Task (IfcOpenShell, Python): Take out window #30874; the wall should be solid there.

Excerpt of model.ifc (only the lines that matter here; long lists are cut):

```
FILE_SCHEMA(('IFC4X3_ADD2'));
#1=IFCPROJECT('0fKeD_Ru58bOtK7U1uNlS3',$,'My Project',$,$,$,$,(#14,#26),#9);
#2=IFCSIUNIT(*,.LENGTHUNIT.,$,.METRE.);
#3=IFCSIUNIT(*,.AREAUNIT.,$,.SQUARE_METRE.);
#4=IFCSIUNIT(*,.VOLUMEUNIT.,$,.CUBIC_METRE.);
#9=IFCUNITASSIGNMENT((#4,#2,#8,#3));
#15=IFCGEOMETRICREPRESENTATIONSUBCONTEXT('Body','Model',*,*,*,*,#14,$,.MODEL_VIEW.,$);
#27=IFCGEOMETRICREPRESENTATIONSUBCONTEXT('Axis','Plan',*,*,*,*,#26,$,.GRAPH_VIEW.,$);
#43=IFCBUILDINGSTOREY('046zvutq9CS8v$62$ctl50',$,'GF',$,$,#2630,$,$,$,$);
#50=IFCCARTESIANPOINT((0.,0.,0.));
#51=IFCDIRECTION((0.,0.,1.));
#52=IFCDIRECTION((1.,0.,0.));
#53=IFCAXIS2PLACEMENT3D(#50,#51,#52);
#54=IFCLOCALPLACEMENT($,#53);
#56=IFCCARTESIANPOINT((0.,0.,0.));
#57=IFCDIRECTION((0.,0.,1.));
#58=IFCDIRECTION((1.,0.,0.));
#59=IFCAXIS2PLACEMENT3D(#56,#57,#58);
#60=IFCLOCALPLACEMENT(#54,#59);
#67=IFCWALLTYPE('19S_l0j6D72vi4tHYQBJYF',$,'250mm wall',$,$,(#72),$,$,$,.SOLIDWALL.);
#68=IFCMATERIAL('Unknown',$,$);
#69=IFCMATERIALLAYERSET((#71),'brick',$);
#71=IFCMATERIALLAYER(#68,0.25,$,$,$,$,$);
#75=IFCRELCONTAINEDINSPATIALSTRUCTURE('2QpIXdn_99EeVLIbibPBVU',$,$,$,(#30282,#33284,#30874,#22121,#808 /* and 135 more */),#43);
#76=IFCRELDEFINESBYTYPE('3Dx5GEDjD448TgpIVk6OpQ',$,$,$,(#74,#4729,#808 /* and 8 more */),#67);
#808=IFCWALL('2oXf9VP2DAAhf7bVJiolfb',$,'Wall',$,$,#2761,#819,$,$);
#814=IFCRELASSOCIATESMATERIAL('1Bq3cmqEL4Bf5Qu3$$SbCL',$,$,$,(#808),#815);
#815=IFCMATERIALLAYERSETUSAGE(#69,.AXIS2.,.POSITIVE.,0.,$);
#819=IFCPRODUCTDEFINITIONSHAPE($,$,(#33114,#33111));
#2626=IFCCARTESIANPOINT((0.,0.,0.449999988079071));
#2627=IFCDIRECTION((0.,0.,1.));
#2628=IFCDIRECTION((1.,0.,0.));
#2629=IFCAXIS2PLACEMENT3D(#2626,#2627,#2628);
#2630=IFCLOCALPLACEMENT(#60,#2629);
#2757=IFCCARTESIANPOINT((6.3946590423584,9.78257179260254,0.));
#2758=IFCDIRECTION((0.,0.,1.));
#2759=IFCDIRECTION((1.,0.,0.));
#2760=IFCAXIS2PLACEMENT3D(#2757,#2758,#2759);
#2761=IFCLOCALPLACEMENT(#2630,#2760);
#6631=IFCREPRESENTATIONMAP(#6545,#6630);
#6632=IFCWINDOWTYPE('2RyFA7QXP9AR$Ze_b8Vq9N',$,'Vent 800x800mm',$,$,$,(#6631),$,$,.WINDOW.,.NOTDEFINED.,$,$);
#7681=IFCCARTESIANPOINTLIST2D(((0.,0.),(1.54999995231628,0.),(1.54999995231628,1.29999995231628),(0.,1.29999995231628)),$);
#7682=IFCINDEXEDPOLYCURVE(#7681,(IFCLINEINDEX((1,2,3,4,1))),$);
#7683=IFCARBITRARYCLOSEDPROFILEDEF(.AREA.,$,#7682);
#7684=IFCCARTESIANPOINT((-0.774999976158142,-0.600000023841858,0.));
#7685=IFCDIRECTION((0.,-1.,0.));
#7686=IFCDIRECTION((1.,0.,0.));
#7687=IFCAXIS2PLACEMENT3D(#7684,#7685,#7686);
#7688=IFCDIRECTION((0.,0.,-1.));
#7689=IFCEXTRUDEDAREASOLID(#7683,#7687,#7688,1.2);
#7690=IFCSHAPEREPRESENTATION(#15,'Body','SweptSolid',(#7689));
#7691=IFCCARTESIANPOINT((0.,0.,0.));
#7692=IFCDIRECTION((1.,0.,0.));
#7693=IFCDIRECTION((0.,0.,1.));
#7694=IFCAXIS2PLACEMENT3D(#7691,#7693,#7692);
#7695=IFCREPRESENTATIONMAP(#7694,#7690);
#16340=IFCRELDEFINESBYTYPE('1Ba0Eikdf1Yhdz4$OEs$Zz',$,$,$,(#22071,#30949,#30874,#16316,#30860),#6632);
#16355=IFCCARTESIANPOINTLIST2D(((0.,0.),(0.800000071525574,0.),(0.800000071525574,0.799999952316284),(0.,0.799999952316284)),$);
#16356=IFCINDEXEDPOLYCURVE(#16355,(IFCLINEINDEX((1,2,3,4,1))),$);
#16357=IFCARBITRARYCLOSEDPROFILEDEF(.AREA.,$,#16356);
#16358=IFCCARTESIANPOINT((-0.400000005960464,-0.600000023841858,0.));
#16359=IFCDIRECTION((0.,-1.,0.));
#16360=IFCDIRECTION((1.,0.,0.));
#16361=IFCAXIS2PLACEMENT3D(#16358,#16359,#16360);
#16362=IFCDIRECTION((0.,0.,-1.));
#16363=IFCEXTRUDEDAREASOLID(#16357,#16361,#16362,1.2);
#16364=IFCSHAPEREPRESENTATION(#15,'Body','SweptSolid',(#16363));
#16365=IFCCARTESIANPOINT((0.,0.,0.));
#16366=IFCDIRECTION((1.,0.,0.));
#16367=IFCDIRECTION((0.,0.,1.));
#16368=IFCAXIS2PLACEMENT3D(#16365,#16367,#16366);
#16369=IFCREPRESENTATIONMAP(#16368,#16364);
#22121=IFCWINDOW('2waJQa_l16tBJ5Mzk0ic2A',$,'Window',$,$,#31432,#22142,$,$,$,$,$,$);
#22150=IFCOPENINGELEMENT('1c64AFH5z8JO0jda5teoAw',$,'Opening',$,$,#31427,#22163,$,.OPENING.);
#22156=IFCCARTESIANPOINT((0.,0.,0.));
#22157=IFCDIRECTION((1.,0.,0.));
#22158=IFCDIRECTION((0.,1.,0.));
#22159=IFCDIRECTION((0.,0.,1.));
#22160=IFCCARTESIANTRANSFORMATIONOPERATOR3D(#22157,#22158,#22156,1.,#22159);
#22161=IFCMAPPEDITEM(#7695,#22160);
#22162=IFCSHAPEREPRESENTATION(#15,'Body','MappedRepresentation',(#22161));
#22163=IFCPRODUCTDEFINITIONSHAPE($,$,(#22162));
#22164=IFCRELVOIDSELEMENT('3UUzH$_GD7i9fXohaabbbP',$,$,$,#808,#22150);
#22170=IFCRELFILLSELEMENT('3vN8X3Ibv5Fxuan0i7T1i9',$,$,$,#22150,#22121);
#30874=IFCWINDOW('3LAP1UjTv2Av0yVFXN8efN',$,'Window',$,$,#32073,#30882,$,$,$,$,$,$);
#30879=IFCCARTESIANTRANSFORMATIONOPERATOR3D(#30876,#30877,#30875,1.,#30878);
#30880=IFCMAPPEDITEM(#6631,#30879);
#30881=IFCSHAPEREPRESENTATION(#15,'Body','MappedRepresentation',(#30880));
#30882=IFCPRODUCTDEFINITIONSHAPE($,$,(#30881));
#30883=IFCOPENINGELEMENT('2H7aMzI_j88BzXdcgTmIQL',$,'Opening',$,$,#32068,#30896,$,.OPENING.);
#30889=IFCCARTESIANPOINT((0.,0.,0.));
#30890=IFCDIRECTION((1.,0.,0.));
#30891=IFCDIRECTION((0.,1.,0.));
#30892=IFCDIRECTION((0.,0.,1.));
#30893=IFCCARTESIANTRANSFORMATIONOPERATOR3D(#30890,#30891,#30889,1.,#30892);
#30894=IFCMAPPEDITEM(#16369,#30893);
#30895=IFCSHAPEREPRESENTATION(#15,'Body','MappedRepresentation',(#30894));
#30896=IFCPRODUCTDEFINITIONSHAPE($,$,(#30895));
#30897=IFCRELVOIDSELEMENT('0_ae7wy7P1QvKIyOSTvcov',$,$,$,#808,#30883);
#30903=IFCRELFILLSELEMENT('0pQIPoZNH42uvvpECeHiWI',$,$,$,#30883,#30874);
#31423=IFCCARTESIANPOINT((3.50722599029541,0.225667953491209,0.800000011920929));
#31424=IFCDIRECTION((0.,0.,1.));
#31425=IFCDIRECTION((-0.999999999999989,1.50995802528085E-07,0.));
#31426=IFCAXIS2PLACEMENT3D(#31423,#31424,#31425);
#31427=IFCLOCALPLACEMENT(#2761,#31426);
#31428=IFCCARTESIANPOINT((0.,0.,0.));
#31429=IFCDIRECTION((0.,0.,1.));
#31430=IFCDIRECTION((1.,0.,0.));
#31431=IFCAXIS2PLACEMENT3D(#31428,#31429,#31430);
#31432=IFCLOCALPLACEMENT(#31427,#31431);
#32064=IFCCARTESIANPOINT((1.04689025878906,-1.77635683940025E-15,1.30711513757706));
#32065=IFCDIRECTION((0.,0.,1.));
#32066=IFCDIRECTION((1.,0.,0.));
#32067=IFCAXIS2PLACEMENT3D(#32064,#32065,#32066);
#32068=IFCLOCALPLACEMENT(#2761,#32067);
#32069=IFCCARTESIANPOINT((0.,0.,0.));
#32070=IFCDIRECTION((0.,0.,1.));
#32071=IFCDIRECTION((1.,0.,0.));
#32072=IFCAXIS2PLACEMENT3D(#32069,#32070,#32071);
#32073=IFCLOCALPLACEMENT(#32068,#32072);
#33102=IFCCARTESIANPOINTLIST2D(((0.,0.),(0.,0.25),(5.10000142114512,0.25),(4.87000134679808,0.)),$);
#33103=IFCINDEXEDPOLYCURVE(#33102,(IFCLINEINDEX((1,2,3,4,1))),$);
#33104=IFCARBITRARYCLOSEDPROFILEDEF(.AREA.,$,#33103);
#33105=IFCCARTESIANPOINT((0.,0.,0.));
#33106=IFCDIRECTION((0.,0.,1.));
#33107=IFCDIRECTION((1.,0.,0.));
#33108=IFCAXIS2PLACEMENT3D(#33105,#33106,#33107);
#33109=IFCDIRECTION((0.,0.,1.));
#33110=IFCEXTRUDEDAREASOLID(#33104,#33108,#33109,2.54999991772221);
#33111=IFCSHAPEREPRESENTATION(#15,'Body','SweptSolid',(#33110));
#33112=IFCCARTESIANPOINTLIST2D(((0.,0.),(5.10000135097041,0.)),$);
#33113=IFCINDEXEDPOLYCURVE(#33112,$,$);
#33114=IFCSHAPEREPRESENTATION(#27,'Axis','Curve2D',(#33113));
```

```python
import ifcopenshell
import ifcopenshell.api.feature
import ifcopenshell.api.root
import ifcopenshell.geom
import ifcopenshell.util.shape

model = ifcopenshell.open("model.ifc")
settings = ifcopenshell.geom.settings()


def volume(element):
    """Net volume in cubic metres, openings subtracted."""
    shape = ifcopenshell.geom.create_shape(settings, element)
    return ifcopenshell.util.shape.get_volume(shape.geometry)


window = model.by_guid("3LAP1UjTv2Av0yVFXN8efN")
opening = window.FillsVoids[0].RelatingOpeningElement
wall = opening.VoidsElements[0].RelatingBuildingElement
before = volume(wall)

ifcopenshell.api.root.remove_product(model, product=window)
ifcopenshell.api.feature.remove_feature(model, feature=opening)

after = volume(wall)

print(f"wall volume {before:.3f} -> {after:.3f} m3")

model.write("model_rev.ifc")
```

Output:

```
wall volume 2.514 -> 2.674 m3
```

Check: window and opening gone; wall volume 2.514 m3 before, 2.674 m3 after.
